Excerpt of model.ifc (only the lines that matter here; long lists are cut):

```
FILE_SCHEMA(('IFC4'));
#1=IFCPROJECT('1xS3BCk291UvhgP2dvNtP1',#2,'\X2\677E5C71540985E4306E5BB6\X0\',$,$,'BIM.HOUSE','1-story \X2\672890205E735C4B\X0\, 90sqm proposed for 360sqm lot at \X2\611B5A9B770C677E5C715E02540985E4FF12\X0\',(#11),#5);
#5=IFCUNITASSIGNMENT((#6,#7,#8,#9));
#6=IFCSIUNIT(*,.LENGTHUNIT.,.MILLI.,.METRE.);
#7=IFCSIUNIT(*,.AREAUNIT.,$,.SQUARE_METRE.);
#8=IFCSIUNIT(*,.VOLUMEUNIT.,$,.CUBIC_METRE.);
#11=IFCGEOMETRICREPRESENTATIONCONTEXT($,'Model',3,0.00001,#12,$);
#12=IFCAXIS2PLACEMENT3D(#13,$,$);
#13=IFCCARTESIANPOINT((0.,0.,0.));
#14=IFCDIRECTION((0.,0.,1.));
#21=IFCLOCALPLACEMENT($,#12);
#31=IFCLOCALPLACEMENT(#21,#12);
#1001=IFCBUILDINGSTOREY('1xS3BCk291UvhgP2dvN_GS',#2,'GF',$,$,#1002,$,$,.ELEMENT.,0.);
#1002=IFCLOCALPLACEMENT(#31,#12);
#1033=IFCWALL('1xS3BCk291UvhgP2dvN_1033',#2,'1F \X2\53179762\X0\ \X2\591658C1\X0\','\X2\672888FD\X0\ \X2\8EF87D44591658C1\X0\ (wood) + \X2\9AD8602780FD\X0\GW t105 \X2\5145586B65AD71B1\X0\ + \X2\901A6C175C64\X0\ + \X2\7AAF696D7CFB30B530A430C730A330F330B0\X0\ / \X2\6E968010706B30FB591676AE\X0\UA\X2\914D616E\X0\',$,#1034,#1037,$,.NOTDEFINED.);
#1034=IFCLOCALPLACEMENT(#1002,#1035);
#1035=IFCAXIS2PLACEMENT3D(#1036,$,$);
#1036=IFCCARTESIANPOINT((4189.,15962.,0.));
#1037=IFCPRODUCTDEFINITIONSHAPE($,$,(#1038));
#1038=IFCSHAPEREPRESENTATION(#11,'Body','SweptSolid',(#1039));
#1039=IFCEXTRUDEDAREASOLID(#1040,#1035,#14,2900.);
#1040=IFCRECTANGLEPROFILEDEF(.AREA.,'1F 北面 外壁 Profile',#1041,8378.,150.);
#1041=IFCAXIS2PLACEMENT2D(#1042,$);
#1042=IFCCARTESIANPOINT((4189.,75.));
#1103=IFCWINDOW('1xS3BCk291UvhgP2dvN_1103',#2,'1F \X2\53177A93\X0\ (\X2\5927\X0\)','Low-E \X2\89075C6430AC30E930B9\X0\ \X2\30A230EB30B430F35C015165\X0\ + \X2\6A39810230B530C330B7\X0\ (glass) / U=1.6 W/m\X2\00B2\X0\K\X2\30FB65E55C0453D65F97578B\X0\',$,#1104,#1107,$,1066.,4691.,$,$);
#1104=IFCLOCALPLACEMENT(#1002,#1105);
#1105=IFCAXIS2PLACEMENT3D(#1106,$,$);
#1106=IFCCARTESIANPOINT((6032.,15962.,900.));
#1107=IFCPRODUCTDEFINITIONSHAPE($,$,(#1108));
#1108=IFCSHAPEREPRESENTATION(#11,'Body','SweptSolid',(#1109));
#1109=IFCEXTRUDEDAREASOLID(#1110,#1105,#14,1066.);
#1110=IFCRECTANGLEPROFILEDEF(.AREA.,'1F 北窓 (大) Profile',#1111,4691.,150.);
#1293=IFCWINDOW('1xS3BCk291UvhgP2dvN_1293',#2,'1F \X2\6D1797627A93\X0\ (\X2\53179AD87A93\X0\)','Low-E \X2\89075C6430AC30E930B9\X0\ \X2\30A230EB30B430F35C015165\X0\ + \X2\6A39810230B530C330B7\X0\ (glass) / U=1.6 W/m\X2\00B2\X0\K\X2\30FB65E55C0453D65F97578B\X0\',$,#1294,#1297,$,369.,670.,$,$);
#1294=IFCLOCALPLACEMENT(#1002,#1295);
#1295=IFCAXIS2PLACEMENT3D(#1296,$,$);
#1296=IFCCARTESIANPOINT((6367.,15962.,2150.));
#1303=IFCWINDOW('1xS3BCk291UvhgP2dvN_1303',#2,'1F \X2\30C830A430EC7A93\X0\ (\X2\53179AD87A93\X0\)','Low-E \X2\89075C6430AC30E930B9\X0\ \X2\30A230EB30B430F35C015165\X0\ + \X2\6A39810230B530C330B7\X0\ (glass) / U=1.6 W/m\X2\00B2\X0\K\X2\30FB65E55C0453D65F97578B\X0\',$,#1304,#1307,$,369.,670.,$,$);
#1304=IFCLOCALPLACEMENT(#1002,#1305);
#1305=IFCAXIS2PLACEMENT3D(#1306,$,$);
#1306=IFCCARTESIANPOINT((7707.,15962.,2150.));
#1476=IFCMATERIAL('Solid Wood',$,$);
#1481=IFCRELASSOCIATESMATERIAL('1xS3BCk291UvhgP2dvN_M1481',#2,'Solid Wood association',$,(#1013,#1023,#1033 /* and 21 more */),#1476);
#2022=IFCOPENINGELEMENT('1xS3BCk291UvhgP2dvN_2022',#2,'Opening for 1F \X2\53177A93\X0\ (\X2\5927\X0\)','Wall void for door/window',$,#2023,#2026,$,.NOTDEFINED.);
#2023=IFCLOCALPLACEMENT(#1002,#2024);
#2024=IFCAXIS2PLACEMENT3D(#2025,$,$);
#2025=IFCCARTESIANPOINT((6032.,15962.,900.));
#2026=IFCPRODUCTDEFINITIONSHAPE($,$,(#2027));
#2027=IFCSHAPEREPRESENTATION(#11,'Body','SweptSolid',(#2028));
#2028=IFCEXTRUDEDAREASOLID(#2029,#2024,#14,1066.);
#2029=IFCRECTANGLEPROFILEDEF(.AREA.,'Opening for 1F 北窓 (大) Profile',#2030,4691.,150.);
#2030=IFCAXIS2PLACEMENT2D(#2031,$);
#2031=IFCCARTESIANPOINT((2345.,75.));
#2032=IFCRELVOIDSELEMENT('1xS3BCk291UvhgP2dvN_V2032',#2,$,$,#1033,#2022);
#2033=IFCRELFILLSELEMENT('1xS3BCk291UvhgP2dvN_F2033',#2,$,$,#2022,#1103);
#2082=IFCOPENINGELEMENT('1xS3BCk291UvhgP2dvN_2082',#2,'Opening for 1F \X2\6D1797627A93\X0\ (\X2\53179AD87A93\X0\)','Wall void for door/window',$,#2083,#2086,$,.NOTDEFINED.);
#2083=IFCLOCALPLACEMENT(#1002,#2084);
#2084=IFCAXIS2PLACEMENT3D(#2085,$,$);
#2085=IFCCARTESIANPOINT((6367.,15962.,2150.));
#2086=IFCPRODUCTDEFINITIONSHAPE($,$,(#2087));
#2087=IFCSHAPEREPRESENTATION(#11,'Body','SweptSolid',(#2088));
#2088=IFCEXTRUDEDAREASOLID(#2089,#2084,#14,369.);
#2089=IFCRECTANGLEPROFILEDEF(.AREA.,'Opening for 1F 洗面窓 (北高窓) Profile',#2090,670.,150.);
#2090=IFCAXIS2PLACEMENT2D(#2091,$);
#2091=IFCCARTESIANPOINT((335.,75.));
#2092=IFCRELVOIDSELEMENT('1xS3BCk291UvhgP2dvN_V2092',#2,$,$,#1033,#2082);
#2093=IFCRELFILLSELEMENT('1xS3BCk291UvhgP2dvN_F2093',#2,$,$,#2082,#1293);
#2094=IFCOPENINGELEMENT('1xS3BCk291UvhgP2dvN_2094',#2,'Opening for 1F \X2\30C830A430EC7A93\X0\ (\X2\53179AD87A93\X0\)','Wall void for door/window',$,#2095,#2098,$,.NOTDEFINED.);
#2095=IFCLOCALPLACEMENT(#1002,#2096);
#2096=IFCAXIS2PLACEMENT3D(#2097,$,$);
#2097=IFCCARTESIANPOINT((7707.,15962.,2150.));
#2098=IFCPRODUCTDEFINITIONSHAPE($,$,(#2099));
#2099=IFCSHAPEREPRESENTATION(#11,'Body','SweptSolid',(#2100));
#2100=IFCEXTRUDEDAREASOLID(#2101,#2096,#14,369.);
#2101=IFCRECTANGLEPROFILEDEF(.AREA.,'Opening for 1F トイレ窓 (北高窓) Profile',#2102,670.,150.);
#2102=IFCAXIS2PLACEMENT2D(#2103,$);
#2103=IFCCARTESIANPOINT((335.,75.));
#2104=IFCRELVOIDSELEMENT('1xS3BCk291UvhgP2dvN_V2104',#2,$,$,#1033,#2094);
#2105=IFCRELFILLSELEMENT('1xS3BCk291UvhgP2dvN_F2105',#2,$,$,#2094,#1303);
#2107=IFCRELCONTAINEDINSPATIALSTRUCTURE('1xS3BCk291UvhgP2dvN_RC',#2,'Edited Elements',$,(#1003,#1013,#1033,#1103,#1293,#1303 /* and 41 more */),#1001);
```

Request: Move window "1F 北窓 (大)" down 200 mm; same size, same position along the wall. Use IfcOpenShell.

```python
import numpy as np
import ifcopenshell
import ifcopenshell.api.geometry
import ifcopenshell.util.placement
import ifcopenshell.util.unit

model = ifcopenshell.open("model.ifc")
unit_scale = ifcopenshell.util.unit.calculate_unit_scale(model)

window = model.by_guid("1xS3BCk291UvhgP2dvN_1103")
opening = window.FillsVoids[0].RelatingOpeningElement
dz = -0.2 / unit_scale

shift = np.array([0.0, 0.0, dz])
# The window is not placed relative to its opening, so move both.
for product in (opening, window):
    matrix = ifcopenshell.util.placement.get_local_placement(product.ObjectPlacement)
    matrix[:3, 3] += shift
    ifcopenshell.api.geometry.edit_object_placement(model, product=product, matrix=matrix, is_si=False)

print(f"moved by {dz * unit_scale:+.3f} m")

model.write("model_v2.ifc")
```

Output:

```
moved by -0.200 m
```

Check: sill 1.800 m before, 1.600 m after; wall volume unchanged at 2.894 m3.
